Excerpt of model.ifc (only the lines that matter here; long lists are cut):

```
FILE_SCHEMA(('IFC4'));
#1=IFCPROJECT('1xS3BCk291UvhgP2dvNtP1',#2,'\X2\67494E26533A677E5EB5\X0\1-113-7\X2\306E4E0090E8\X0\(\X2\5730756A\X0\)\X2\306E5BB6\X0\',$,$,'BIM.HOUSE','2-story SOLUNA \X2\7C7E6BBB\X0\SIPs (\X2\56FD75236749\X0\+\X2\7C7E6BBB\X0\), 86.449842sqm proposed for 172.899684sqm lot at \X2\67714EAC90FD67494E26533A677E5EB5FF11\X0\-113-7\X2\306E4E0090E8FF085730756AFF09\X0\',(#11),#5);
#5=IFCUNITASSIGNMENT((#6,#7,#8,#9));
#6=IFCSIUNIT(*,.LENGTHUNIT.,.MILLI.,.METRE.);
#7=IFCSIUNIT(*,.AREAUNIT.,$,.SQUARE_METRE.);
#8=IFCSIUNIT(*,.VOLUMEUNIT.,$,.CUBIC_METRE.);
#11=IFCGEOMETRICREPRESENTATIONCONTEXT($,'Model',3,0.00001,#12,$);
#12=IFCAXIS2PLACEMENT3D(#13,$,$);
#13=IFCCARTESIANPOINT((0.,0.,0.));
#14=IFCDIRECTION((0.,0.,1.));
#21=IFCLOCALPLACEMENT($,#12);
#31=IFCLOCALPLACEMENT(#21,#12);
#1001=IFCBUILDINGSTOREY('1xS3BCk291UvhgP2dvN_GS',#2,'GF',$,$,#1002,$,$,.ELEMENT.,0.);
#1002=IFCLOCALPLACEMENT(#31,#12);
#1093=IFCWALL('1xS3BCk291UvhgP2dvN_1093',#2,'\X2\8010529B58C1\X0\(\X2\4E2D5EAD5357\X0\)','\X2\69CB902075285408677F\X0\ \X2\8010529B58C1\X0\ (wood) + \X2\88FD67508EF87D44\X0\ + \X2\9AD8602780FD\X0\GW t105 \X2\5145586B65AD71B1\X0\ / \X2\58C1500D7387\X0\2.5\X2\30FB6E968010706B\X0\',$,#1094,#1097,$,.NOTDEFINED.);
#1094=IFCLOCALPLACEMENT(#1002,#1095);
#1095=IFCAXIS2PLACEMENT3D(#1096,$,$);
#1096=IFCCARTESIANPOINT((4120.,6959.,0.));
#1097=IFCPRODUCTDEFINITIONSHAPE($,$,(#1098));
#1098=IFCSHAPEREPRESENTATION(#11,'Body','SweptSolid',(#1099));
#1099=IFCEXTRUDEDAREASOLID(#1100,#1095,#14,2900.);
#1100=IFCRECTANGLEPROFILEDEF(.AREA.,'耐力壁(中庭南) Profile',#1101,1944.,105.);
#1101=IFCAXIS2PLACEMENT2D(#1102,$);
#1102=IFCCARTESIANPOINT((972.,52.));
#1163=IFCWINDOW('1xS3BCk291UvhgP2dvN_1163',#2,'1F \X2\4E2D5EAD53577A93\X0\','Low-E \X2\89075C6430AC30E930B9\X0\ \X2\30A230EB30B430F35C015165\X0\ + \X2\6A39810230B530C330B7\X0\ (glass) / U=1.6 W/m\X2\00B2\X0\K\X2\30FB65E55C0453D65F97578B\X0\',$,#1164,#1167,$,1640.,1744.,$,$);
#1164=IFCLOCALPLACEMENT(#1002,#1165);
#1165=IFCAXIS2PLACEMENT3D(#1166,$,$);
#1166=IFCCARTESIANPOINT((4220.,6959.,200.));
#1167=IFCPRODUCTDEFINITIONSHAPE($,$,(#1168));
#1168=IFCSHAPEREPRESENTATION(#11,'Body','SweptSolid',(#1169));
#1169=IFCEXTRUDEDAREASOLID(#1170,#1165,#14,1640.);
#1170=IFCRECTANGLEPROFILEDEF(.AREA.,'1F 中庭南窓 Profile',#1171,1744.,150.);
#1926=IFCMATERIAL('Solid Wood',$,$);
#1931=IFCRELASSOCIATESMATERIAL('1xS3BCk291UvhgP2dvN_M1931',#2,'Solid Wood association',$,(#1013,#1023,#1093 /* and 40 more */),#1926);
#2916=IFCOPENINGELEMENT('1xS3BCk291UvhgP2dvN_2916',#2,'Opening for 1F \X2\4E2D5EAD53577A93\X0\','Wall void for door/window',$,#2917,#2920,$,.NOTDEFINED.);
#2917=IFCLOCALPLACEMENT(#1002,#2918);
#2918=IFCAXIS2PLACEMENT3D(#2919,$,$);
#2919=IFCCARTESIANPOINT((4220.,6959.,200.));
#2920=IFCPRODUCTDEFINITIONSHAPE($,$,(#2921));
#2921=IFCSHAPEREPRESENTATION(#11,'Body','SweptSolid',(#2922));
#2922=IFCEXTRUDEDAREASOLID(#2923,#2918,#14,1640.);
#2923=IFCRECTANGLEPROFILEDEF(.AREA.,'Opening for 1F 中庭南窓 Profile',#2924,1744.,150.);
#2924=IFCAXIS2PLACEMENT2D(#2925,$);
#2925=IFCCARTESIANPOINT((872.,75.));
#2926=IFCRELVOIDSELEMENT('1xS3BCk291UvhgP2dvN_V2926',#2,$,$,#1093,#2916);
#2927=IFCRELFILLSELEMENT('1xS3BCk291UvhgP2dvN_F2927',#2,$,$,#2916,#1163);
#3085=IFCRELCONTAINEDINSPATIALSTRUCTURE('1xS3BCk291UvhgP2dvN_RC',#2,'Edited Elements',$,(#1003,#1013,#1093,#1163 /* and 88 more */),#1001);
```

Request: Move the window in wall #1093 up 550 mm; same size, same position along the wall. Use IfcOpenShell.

```python
import numpy as np
import ifcopenshell
import ifcopenshell.api.geometry
import ifcopenshell.util.placement
import ifcopenshell.util.unit

model = ifcopenshell.open("model.ifc")
unit_scale = ifcopenshell.util.unit.calculate_unit_scale(model)

window = model.by_id(1163)
opening = window.FillsVoids[0].RelatingOpeningElement
dz = 0.55 / unit_scale

shift = np.array([0.0, 0.0, dz])
# The window is not placed relative to its opening, so move both.
for product in (opening, window):
    matrix = ifcopenshell.util.placement.get_local_placement(product.ObjectPlacement)
    matrix[:3, 3] += shift
    ifcopenshell.api.geometry.edit_object_placement(model, product=product, matrix=matrix, is_si=False)

print(f"moved by {dz * unit_scale:+.3f} m")

model.write("model_v2.ifc")
```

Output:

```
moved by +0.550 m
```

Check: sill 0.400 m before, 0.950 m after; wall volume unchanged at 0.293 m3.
